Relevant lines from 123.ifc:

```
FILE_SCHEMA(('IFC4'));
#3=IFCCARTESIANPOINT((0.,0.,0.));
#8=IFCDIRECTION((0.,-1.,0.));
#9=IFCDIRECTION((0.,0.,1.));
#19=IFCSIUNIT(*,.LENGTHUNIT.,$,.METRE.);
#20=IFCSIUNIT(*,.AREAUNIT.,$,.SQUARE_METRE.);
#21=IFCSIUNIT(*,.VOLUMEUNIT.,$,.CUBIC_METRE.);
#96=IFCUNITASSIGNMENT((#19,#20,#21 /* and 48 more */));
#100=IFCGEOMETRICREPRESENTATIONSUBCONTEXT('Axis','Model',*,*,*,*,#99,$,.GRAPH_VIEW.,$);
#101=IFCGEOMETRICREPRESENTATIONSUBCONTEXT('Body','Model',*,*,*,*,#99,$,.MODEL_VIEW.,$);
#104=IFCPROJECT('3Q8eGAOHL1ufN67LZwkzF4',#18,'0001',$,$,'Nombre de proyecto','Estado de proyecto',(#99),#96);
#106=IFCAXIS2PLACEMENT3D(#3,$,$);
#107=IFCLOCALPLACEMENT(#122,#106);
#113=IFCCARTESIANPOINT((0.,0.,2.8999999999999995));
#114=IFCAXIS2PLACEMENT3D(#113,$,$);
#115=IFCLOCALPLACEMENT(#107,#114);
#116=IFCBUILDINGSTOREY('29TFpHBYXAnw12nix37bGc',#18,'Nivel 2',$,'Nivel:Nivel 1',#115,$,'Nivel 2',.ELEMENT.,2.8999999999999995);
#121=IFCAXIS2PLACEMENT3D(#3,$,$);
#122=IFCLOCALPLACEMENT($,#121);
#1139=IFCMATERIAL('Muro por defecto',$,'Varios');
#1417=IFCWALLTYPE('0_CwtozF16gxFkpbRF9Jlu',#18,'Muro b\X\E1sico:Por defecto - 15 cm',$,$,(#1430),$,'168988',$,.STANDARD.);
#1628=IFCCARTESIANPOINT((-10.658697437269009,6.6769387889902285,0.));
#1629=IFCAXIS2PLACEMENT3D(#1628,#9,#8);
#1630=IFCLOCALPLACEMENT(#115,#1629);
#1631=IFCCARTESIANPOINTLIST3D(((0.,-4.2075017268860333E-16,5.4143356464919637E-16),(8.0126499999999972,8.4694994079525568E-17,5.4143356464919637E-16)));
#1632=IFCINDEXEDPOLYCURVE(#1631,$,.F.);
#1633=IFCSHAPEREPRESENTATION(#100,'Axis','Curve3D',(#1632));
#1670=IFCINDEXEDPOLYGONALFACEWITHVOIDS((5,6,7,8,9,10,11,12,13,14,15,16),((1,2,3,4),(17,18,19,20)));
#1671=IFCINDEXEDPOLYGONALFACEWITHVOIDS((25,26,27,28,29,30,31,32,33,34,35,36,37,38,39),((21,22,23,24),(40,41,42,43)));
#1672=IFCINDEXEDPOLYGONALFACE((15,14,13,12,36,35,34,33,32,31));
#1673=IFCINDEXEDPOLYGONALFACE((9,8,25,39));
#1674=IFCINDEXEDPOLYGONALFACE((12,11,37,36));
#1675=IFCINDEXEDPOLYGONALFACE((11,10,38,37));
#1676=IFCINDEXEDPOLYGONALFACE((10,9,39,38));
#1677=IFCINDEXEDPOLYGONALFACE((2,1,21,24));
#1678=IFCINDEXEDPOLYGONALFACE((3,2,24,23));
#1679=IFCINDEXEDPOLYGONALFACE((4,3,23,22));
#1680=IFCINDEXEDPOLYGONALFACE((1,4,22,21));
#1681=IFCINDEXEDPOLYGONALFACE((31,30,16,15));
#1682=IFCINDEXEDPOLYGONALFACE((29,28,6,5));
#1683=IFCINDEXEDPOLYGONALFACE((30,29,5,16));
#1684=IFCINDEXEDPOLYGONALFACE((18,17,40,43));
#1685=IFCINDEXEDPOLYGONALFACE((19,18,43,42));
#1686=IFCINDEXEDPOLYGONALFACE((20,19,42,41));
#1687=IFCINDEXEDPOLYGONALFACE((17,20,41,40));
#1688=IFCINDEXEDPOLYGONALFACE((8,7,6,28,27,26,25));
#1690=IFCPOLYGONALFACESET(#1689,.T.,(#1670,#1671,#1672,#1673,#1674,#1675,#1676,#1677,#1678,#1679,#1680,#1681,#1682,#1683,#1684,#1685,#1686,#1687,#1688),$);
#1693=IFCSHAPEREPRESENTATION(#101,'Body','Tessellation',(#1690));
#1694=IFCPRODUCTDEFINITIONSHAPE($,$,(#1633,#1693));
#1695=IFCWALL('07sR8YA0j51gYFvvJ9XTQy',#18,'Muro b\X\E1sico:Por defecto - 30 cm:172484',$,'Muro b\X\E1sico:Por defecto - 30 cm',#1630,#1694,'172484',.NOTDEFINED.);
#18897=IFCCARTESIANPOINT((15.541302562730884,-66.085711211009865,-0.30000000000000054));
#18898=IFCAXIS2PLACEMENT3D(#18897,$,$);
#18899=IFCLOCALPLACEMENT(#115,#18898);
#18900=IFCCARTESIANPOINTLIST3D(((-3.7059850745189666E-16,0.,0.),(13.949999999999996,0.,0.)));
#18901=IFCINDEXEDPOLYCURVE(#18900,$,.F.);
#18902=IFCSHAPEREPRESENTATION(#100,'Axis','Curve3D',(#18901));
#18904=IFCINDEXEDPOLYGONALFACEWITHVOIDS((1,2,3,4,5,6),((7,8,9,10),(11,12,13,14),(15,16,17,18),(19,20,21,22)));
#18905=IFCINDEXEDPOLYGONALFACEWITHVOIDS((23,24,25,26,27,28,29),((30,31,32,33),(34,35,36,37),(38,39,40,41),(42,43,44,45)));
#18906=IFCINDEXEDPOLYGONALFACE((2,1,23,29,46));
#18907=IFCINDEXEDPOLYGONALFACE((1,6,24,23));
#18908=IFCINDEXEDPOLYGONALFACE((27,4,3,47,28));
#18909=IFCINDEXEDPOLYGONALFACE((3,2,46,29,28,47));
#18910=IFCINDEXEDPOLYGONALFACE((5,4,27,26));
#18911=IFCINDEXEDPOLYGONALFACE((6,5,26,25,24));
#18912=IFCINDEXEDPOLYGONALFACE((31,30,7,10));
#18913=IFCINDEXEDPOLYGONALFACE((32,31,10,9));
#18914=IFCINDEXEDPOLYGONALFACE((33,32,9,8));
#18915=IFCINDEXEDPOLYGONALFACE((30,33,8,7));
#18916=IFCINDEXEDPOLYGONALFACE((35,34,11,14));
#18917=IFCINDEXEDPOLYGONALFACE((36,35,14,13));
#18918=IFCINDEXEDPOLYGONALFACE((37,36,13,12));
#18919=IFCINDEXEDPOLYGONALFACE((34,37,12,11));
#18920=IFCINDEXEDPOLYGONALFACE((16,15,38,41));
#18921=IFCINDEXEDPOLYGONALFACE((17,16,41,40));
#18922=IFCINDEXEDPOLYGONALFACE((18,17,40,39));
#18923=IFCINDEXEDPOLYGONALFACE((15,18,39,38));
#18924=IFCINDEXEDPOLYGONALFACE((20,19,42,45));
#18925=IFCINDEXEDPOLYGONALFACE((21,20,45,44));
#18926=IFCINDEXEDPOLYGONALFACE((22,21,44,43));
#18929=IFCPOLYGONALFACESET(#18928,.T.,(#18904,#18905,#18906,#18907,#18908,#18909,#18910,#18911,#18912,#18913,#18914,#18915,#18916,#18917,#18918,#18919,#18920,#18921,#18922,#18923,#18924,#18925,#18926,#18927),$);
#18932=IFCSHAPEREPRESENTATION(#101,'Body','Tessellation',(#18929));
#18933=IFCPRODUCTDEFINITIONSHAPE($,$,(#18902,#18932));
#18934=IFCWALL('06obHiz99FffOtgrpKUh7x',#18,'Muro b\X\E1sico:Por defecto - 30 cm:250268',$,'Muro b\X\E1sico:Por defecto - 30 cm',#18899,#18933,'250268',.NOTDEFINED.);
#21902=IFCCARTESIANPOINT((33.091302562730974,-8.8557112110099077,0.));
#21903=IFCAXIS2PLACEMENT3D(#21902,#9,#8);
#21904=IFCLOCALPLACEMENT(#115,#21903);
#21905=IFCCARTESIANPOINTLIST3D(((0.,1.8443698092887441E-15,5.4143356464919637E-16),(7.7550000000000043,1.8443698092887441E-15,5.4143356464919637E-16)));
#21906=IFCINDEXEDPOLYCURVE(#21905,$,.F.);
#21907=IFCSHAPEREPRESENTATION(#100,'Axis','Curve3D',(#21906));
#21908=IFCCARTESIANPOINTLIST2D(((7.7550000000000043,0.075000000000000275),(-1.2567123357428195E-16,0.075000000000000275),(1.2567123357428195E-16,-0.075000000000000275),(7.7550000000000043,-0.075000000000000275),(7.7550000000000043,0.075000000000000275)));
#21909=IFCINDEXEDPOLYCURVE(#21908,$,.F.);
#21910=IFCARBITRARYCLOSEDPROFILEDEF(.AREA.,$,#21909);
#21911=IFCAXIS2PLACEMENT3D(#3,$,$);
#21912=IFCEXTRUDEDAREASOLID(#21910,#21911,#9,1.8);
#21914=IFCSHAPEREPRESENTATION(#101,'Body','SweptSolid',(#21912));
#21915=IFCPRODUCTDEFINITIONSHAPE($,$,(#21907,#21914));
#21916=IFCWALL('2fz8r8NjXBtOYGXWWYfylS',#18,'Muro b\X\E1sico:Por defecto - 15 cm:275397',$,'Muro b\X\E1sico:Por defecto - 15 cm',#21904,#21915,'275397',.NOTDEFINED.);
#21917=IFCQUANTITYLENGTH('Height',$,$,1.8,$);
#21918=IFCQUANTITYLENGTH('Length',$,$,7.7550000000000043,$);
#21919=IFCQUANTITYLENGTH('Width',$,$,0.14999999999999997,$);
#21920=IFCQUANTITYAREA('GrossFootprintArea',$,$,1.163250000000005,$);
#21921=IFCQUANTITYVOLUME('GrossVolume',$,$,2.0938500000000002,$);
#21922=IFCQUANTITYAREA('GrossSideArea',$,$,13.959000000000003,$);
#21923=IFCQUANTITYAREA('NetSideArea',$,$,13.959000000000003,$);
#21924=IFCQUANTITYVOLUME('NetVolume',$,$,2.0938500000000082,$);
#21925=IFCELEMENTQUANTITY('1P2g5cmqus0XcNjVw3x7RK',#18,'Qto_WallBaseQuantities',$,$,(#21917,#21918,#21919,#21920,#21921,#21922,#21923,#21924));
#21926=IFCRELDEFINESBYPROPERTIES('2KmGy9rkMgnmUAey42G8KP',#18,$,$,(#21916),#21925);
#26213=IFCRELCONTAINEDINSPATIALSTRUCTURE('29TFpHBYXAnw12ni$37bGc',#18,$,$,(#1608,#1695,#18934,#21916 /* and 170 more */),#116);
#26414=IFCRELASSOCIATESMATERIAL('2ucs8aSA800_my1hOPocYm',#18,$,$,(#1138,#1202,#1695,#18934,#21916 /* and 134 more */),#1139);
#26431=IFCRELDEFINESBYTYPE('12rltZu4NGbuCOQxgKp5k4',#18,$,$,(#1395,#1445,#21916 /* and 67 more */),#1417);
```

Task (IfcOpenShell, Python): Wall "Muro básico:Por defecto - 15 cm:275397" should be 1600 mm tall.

```python
import ifcopenshell
import ifcopenshell.api.pset
import ifcopenshell.geom
import ifcopenshell.util.element
import ifcopenshell.util.representation
import ifcopenshell.util.shape
import ifcopenshell.util.unit

model = ifcopenshell.open("123.ifc")
unit_scale = ifcopenshell.util.unit.calculate_unit_scale(model)
area_scale = ifcopenshell.util.unit.calculate_unit_scale(model, "AREAUNIT")
volume_scale = ifcopenshell.util.unit.calculate_unit_scale(model, "VOLUMEUNIT")
settings = ifcopenshell.geom.settings()


def volume(element):
    """Net volume in cubic metres, openings subtracted."""
    shape = ifcopenshell.geom.create_shape(settings, element)
    return ifcopenshell.util.shape.get_volume(shape.geometry)


wall = model.by_guid("2fz8r8NjXBtOYGXWWYfylS")
before = volume(wall)

body = ifcopenshell.util.representation.get_representation(wall, "Model", "Body")
solid = body.Items[0]
old_height = solid.Depth
solid.Depth = 1.6 / unit_scale
after = volume(wall)
thickness = 0.15  # wall thickness in metres

# Update the stored height, areas and volumes.
qto = model.by_id(ifcopenshell.util.element.get_pset(wall, "Qto_WallBaseQuantities", should_inherit=False)["id"])
ifcopenshell.api.pset.edit_qto(model, qto=qto, properties={
    "Height": solid.Depth,
    "GrossVolume": ifcopenshell.util.element.get_pset(wall, "Qto_WallBaseQuantities", "GrossVolume") * solid.Depth / old_height,
    "GrossSideArea": ifcopenshell.util.element.get_pset(wall, "Qto_WallBaseQuantities", "GrossSideArea") * solid.Depth / old_height,
    "NetSideArea": after / thickness / area_scale,
    "NetVolume": after / volume_scale,
})

print(f"height {old_height:g} -> {solid.Depth:g}, volume {before:.3f} -> {after:.3f} m3")

model.write("123-out.ifc")
```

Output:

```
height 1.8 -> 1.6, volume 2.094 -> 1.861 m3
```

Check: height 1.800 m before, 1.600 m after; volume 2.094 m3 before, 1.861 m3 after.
